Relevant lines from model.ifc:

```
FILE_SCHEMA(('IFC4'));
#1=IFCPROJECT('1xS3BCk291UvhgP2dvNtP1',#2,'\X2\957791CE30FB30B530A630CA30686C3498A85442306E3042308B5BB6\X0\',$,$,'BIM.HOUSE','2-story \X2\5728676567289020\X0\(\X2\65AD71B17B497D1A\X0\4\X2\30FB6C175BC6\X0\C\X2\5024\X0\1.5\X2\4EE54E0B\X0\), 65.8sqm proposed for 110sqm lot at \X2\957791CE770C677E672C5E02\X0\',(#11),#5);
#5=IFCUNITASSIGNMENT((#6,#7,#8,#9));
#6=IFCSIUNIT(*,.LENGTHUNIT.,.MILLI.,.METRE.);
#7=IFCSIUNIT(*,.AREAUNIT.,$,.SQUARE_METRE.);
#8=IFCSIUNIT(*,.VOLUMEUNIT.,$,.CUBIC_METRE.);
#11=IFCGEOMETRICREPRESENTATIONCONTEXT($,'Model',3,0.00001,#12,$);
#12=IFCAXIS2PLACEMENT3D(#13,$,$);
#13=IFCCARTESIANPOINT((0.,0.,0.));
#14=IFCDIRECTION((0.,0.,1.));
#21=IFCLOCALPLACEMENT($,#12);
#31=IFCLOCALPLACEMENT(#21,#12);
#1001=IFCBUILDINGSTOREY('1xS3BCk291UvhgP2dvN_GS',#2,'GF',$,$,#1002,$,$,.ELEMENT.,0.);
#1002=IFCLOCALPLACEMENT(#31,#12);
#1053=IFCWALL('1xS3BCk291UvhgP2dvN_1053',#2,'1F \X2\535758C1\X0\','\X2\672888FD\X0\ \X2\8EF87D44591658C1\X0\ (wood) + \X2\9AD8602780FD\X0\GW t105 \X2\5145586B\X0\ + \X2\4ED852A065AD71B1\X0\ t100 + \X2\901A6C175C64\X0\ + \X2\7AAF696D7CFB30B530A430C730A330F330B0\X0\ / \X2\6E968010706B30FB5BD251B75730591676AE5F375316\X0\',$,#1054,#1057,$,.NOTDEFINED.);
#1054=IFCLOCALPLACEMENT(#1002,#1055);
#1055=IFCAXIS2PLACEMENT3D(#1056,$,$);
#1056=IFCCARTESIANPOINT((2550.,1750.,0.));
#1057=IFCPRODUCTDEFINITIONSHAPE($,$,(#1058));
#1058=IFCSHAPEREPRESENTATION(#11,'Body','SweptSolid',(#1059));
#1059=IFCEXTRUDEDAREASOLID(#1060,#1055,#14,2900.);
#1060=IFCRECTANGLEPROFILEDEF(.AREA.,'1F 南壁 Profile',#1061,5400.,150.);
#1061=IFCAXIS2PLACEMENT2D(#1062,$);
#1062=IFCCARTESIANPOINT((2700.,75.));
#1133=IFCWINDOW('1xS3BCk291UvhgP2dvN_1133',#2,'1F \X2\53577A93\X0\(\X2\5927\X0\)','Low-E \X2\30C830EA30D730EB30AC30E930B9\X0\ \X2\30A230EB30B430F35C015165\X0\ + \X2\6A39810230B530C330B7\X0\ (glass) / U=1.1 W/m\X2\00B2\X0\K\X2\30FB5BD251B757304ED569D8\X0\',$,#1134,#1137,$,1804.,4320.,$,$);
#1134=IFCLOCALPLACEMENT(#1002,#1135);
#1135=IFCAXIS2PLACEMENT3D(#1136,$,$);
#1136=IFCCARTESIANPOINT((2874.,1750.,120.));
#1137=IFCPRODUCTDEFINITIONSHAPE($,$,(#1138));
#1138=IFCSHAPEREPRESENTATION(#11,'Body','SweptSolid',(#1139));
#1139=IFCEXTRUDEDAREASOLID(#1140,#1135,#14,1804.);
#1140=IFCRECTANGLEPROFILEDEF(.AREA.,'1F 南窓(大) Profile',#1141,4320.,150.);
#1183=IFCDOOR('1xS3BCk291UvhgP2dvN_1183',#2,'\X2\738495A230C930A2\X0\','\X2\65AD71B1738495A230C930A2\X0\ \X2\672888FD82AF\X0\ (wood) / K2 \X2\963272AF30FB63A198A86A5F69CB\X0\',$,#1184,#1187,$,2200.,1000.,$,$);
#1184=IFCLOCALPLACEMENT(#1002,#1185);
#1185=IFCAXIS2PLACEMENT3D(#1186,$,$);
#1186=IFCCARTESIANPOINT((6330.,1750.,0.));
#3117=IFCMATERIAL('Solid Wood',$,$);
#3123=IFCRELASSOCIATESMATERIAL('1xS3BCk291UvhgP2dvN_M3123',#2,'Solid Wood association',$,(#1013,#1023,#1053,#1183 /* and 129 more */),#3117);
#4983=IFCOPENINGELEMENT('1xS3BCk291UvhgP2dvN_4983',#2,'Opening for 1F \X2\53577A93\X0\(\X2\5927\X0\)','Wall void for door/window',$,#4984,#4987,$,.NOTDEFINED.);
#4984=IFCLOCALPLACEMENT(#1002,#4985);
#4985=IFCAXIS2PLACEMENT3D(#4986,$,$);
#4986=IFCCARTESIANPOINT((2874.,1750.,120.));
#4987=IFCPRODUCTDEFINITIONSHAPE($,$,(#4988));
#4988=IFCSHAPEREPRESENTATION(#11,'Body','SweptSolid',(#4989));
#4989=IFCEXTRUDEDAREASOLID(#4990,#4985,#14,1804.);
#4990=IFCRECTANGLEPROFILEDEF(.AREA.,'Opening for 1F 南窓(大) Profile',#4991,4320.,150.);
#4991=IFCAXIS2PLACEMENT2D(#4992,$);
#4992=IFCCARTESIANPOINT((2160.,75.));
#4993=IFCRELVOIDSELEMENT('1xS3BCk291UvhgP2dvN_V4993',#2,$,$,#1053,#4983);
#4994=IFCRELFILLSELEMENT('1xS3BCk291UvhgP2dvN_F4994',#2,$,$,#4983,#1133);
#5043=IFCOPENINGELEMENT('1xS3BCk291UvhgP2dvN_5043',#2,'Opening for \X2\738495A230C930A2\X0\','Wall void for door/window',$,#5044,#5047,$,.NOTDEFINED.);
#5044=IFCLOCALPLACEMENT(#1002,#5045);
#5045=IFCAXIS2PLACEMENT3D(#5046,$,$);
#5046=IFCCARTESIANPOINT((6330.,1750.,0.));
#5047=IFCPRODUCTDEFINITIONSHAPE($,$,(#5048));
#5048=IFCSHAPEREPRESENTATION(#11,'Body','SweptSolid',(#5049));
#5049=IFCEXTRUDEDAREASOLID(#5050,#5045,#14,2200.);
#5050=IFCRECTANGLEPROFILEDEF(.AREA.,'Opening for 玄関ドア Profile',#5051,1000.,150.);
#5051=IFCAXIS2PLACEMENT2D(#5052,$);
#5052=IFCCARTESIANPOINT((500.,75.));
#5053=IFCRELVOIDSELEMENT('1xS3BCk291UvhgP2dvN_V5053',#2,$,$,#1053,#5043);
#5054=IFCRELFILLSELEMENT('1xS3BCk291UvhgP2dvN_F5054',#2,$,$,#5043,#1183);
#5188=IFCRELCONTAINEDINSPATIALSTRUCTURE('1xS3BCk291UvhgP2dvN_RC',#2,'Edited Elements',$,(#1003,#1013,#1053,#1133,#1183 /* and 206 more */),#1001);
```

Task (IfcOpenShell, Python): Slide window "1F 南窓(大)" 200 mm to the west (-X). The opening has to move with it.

```python
import ifcopenshell
import ifcopenshell.api.geometry
import ifcopenshell.util.placement

model = ifcopenshell.open("model.ifc")

window = model.by_id(1133)
opening = window.FillsVoids[0].RelatingOpeningElement
wall = opening.VoidsElements[0].RelatingBuildingElement

wall_matrix = ifcopenshell.util.placement.get_local_placement(wall.ObjectPlacement)
shift = wall_matrix[:3, 0] * -200.0
before = ifcopenshell.util.placement.get_local_placement(window.ObjectPlacement)[:3, 3].copy()

# The window is not placed relative to its opening, so move both.
for product in (opening, window):
    matrix = ifcopenshell.util.placement.get_local_placement(product.ObjectPlacement)
    matrix[:3, 3] += shift
    ifcopenshell.api.geometry.edit_object_placement(model, product=product, matrix=matrix, is_si=False)

after = ifcopenshell.util.placement.get_local_placement(window.ObjectPlacement)[:3, 3]
print("window moved by", (after - before).round(3) + 0.0)

model.write("model_rev.ifc")
```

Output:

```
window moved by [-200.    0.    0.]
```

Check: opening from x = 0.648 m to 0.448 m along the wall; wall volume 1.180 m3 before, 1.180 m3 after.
